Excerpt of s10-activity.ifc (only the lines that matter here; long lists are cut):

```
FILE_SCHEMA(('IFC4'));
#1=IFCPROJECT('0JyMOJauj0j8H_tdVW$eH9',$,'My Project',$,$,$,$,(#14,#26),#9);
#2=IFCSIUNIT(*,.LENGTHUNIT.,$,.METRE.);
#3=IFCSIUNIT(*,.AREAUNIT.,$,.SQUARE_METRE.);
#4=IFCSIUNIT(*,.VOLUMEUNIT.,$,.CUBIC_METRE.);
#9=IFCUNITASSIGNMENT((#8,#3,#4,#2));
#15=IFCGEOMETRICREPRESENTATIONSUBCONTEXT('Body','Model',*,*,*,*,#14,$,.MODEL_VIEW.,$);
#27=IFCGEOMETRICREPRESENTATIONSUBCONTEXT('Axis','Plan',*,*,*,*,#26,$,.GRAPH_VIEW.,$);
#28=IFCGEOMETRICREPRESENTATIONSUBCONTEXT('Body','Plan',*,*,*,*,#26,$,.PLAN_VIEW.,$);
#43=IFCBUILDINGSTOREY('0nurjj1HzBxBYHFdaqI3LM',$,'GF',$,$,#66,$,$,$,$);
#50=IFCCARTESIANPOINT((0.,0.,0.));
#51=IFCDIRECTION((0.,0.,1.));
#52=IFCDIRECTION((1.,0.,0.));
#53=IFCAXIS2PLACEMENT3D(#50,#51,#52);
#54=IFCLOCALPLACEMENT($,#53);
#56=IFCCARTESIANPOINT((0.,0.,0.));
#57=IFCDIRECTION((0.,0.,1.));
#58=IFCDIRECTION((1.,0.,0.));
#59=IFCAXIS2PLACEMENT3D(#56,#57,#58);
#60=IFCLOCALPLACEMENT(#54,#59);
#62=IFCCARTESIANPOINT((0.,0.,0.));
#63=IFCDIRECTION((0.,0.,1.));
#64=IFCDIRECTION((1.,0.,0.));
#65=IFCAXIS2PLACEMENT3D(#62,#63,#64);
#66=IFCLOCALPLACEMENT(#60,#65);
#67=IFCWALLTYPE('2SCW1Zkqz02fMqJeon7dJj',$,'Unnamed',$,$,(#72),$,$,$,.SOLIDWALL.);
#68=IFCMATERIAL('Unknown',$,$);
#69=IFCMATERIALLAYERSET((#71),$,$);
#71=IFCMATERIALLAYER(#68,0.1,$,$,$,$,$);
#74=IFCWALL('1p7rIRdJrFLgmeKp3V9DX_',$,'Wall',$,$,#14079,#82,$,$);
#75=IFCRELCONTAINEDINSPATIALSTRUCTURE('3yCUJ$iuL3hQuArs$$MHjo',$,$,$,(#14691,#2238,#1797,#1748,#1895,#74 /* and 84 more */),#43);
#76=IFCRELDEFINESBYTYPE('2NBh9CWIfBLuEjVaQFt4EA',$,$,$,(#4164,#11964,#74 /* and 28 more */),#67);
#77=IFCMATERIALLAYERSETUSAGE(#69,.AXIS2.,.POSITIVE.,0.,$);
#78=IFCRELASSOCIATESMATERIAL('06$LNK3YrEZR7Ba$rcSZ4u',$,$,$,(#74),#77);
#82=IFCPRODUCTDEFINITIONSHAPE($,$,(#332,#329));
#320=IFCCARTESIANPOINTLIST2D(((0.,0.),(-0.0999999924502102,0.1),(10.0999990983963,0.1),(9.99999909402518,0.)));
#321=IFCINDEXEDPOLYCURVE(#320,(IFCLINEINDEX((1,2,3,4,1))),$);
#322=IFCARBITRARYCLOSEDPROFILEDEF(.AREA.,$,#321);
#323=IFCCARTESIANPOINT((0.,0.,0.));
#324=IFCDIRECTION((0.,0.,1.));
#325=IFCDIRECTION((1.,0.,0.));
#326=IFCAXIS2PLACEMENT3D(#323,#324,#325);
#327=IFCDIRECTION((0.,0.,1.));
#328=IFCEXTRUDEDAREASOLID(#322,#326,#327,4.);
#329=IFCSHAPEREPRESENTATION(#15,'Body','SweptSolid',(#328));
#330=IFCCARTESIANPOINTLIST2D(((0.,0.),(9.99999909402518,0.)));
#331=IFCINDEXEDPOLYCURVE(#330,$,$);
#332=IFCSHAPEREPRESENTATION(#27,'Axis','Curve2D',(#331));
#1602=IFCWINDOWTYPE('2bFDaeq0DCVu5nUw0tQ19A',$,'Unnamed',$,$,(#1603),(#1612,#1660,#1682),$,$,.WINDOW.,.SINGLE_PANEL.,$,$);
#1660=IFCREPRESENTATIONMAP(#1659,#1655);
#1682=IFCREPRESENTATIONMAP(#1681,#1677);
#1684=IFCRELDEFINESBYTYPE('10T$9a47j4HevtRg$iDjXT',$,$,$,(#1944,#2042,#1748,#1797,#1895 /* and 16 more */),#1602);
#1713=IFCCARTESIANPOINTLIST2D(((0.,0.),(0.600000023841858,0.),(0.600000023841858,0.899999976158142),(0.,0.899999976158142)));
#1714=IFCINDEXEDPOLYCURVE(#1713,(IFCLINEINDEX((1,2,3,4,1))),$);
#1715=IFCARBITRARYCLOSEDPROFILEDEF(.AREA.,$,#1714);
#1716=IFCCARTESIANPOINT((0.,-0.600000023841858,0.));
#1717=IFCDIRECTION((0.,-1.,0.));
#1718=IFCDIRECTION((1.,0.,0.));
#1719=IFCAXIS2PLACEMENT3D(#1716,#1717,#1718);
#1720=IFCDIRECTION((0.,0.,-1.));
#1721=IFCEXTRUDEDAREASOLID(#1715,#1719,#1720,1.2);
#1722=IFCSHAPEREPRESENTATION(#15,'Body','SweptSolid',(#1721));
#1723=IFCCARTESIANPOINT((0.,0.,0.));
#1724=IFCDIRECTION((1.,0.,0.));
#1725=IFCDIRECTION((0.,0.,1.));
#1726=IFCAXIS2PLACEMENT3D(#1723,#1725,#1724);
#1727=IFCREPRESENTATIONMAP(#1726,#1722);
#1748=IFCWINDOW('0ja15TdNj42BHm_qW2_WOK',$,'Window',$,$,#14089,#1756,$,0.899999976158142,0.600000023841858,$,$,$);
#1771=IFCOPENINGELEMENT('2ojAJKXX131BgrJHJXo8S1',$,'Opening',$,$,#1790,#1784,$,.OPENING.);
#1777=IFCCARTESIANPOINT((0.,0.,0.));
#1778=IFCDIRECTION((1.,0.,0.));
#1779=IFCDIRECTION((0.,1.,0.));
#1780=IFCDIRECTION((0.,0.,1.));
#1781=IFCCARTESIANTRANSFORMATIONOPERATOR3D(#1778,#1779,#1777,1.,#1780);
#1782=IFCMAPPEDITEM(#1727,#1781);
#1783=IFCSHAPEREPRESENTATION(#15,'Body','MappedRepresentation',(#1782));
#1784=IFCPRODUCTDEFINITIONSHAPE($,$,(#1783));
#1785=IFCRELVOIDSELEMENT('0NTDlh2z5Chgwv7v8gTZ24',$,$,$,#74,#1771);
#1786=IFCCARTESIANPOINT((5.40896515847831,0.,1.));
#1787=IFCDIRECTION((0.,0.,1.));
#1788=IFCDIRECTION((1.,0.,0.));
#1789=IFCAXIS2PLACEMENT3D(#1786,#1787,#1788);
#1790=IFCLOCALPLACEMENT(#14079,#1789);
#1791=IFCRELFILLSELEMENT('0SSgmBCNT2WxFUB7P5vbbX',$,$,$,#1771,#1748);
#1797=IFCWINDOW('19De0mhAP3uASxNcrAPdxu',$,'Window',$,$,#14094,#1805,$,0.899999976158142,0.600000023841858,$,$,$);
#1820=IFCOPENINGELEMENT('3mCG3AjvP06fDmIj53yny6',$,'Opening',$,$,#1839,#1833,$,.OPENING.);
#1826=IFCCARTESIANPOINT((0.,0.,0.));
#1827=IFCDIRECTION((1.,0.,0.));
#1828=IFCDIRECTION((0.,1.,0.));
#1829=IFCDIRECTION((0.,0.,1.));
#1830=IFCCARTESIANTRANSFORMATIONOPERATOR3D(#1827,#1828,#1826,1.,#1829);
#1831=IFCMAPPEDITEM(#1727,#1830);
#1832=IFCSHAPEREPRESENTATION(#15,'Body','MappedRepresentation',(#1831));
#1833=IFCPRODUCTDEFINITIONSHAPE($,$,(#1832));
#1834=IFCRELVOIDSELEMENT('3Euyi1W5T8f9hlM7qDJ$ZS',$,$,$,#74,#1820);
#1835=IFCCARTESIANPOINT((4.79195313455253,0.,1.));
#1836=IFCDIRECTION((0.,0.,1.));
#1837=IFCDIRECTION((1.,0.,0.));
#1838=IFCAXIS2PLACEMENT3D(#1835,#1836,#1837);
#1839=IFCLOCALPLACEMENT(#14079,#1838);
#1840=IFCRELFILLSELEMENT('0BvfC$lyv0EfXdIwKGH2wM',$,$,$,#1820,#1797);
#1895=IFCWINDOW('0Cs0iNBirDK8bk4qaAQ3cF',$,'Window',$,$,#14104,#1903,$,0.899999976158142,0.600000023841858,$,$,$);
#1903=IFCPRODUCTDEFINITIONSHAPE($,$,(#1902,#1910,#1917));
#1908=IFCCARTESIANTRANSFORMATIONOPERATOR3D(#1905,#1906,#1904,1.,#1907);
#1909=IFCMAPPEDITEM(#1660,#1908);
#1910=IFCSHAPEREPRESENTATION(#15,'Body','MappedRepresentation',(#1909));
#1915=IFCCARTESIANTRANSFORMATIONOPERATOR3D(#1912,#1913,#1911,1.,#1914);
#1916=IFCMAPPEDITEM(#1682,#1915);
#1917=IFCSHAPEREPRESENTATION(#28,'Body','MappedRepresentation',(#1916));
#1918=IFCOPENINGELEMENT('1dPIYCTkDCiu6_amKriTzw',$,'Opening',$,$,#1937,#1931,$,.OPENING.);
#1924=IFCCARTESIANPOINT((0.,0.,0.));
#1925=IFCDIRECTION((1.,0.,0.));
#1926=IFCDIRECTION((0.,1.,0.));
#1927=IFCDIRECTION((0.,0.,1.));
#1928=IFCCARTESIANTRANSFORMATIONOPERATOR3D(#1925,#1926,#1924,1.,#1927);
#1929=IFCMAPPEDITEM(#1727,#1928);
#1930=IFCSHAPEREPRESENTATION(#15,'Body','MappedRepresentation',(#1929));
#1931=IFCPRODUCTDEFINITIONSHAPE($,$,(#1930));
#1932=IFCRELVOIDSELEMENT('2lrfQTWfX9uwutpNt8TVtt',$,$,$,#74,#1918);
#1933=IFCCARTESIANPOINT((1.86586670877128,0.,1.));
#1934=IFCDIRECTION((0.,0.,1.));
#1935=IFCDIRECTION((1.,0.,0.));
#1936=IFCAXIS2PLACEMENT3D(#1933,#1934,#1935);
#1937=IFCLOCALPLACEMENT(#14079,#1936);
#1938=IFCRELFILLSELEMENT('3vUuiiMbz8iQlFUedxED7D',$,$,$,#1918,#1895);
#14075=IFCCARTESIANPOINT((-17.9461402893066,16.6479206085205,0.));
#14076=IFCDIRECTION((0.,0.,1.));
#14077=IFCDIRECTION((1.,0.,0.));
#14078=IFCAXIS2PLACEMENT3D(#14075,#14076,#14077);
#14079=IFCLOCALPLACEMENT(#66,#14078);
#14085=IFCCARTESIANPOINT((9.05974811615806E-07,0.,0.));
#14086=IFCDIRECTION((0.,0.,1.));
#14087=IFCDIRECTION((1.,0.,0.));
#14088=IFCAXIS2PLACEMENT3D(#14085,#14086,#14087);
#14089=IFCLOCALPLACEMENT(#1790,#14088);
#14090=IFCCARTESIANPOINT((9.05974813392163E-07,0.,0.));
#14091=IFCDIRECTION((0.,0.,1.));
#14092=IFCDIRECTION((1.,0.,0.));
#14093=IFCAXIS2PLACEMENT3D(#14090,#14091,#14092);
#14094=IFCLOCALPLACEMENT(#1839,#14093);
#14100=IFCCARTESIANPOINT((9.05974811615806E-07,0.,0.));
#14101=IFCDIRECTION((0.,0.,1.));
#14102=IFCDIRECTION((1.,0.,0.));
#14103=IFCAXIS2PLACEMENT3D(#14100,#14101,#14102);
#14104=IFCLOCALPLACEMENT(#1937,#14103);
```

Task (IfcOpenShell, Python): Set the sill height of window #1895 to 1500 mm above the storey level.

```python
import numpy as np
import ifcopenshell
import ifcopenshell.api.geometry
import ifcopenshell.geom
import ifcopenshell.util.element
import ifcopenshell.util.placement
import ifcopenshell.util.shape
import ifcopenshell.util.unit

model = ifcopenshell.open("s10-activity.ifc")
unit_scale = ifcopenshell.util.unit.calculate_unit_scale(model)

window = model.by_guid("0Cs0iNBirDK8bk4qaAQ3cF")
opening = window.FillsVoids[0].RelatingOpeningElement
storey = ifcopenshell.util.element.get_container(window, ifc_class="IfcBuildingStorey")
level = ifcopenshell.util.placement.get_local_placement(storey.ObjectPlacement)[2, 3]

# The opening's origin need not be at the sill, so measure its lowest point.
shape = ifcopenshell.geom.create_shape(ifcopenshell.geom.settings(), opening)
bottom = ifcopenshell.util.shape.get_shape_bottom_elevation(shape, shape.geometry) / unit_scale
dz = level + 1.5 - bottom

shift = np.array([0.0, 0.0, dz])
# The window is placed relative to its opening, so it follows when the opening moves.
matrix = ifcopenshell.util.placement.get_local_placement(opening.ObjectPlacement)
matrix[:3, 3] += shift
ifcopenshell.api.geometry.edit_object_placement(
    model, product=opening, matrix=matrix, is_si=False, should_transform_children=True
)

print(f"moved by {dz * unit_scale:+.3f} m")

model.write("s10-activity_updated.ifc")
```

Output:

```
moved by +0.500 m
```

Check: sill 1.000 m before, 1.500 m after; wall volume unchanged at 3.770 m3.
